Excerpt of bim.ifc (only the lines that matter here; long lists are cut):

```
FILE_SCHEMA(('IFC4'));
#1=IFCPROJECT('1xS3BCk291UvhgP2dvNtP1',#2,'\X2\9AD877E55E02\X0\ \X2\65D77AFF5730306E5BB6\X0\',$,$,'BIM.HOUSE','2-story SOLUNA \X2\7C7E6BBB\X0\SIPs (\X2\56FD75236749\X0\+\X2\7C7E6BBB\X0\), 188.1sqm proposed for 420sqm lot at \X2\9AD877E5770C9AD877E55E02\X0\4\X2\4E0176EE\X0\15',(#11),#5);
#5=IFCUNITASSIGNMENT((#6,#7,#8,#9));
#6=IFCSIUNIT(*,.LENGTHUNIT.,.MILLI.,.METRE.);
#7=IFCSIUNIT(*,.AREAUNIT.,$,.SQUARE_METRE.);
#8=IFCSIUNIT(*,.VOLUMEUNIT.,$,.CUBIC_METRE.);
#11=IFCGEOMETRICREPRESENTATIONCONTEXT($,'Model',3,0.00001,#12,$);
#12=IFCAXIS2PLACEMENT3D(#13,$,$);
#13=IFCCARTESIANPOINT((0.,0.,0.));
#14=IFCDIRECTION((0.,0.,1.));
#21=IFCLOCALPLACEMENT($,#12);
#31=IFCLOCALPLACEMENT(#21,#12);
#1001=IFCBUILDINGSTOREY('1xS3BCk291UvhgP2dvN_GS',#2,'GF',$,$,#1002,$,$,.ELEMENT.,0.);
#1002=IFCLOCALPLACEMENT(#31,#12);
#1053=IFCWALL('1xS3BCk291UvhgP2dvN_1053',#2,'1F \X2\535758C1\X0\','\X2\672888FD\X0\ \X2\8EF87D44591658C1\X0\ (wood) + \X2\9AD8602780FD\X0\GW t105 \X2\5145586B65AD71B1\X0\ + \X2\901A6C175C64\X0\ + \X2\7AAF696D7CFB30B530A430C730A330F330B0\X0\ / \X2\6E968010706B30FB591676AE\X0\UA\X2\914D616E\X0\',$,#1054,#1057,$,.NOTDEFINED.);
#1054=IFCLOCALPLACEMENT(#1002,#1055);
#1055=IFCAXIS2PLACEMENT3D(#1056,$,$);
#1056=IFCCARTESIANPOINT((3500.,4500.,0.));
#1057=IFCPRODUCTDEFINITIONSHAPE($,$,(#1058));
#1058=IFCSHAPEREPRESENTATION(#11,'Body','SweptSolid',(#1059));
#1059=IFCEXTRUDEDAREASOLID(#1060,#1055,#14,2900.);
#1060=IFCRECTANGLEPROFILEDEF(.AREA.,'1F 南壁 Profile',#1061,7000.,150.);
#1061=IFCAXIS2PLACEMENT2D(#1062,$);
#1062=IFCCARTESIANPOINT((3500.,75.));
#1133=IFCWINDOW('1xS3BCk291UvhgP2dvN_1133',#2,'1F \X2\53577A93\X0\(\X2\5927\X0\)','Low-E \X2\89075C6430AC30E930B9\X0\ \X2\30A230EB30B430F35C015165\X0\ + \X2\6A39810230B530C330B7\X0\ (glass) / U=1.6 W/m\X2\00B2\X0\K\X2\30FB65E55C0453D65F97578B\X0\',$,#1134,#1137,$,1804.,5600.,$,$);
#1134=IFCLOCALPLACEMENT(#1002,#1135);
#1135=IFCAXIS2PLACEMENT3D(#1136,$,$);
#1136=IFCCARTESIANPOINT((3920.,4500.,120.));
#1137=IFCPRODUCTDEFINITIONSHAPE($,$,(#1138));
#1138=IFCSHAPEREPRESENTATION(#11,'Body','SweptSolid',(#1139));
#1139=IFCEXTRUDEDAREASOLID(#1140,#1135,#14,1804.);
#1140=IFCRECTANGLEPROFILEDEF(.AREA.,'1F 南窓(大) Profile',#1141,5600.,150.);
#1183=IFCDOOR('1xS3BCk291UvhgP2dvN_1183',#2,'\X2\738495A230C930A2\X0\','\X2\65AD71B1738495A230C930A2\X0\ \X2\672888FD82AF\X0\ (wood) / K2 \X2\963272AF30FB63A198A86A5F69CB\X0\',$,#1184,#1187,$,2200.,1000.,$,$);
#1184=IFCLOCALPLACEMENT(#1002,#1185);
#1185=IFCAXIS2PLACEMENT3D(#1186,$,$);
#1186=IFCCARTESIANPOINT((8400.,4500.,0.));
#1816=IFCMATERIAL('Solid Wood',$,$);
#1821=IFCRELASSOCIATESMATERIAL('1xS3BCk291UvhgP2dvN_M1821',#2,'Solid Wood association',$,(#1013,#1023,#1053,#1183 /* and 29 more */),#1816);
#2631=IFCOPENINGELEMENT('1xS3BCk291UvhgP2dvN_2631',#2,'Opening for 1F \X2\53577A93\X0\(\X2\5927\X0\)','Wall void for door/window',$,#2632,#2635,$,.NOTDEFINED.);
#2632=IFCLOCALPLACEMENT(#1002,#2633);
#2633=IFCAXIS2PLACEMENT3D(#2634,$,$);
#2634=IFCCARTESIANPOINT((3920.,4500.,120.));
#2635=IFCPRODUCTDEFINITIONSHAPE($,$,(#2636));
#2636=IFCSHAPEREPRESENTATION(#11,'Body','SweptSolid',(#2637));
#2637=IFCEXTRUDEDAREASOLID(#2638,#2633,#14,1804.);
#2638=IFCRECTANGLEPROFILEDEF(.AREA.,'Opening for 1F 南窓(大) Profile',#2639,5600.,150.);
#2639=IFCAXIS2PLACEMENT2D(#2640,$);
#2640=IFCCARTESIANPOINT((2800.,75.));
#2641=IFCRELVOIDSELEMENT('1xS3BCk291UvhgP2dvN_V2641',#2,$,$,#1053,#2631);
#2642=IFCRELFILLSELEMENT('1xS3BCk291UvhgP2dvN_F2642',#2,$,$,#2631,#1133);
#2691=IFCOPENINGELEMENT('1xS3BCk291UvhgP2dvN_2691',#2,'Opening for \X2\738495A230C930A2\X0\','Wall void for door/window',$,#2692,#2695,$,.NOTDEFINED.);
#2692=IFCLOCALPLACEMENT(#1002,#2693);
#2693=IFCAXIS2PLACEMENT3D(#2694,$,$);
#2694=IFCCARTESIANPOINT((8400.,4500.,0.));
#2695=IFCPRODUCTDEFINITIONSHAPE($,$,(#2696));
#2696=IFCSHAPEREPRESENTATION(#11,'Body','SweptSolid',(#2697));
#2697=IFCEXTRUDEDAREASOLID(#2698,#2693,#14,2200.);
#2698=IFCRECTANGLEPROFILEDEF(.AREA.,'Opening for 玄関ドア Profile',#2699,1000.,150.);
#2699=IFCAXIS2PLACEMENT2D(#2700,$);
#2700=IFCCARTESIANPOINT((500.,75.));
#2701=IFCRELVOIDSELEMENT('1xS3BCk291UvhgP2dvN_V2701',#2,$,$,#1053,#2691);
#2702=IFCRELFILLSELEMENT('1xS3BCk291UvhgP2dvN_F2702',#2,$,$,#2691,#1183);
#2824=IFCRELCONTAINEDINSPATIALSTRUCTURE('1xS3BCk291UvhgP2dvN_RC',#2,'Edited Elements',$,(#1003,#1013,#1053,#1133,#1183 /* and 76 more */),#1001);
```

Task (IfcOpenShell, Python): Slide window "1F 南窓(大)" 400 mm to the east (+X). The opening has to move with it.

```python
import ifcopenshell
import ifcopenshell.api.geometry
import ifcopenshell.util.placement
import ifcopenshell.util.unit

model = ifcopenshell.open("bim.ifc")
unit_scale = ifcopenshell.util.unit.calculate_unit_scale(model)

window = model.by_guid("1xS3BCk291UvhgP2dvN_1133")
opening = window.FillsVoids[0].RelatingOpeningElement
wall = opening.VoidsElements[0].RelatingBuildingElement

wall_matrix = ifcopenshell.util.placement.get_local_placement(wall.ObjectPlacement)
shift = wall_matrix[:3, 0] * 0.4 / unit_scale
before = ifcopenshell.util.placement.get_local_placement(window.ObjectPlacement)[:3, 3].copy()

# The window is not placed relative to its opening, so move both.
for product in (opening, window):
    matrix = ifcopenshell.util.placement.get_local_placement(product.ObjectPlacement)
    matrix[:3, 3] += shift
    ifcopenshell.api.geometry.edit_object_placement(model, product=product, matrix=matrix, is_si=False)

after = ifcopenshell.util.placement.get_local_placement(window.ObjectPlacement)[:3, 3]
print("window moved by", (after - before).round(3) + 0.0)

model.write("bim_v2.ifc")
```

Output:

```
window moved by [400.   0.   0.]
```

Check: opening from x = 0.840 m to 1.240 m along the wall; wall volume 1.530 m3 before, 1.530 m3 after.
